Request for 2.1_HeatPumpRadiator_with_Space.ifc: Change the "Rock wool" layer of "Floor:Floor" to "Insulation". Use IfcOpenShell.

First a look at what the model holds.

```python
import ifcopenshell
import ifcopenshell.util.element

model = ifcopenshell.open("2.1_HeatPumpRadiator_with_Space.ifc")
print(model.schema)
for layer_set in model.by_type("IfcMaterialLayerSet"):
    if layer_set.LayerSetName == "Floor:Floor":
        for layer in layer_set.MaterialLayers:
            print(layer.id(), layer.Material and layer.Material.Name, layer.LayerThickness, sep=" | ")
        print(len(ifcopenshell.util.element.get_elements_by_material(model, layer_set)), "elements and types use it")
print(sorted(m.Name for m in model.by_type("IfcMaterial") if m.Name)[:60])
```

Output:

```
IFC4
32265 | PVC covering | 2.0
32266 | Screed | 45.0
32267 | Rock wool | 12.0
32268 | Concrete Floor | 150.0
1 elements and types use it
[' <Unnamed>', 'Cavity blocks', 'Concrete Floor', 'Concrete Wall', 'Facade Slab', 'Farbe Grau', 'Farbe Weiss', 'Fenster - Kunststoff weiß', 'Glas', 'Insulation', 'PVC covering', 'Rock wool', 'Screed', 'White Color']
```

```python
import ifcopenshell
import ifcopenshell.api.material

model = ifcopenshell.open("2.1_HeatPumpRadiator_with_Space.ifc")

layer_set = next(s for s in model.by_type("IfcMaterialLayerSet") if s.LayerSetName == "Floor:Floor")
layer = next(l for l in layer_set.MaterialLayers if l.Material and l.Material.Name == "Rock wool")
material = next(m for m in model.by_type("IfcMaterial") if m.Name == "Insulation")

# Point this one layer at the other material; renaming the old one would change it everywhere.
ifcopenshell.api.material.edit_layer(model, layer=layer, attributes={}, material=material)

print([l.Material.Name if l.Material else None for l in layer_set.MaterialLayers])

model.write("2.1_HeatPumpRadiator_with_Space_updated.ifc")
```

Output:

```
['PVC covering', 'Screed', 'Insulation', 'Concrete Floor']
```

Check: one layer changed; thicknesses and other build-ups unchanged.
